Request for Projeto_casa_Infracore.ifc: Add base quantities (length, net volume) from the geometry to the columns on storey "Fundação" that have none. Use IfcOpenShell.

First a look at what the model holds.

```python
import ifcopenshell
import ifcopenshell.util.element
import ifcopenshell.util.unit

model = ifcopenshell.open("Projeto_casa_Infracore.ifc")
print(model.schema)
for unit_type in ("LENGTHUNIT", "AREAUNIT", "VOLUMEUNIT"):
    print(unit_type, ifcopenshell.util.unit.calculate_unit_scale(model, unit_type))
storey = next(s for s in model.by_type("IfcBuildingStorey") if s.Name == "Fundação")
columns = [e for e in ifcopenshell.util.element.get_decomposition(storey) if e.is_a("IfcColumn")]
for e in sorted(columns, key=lambda e: e.id()):
    print(e.id(), e.is_a(), e.Name, list(ifcopenshell.util.element.get_psets(e, qtos_only=True)), sep=" | ")
```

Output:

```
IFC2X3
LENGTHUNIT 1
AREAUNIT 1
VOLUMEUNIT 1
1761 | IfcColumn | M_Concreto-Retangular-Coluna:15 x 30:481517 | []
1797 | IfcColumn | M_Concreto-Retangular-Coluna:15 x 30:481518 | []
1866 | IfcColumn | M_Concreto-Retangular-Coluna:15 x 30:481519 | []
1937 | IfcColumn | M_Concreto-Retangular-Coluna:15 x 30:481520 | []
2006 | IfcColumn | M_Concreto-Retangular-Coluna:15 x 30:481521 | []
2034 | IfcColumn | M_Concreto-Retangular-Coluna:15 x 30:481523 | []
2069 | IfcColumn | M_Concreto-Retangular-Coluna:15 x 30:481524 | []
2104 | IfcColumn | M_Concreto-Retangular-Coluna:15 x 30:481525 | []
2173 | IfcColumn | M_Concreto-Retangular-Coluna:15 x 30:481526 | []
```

```python
import ifcopenshell
import ifcopenshell.api.pset
import ifcopenshell.geom
import ifcopenshell.util.element
import ifcopenshell.util.shape
import ifcopenshell.util.unit

model = ifcopenshell.open("Projeto_casa_Infracore.ifc")
unit_scale = ifcopenshell.util.unit.calculate_unit_scale(model)
volume_scale = ifcopenshell.util.unit.calculate_unit_scale(model, "VOLUMEUNIT")
settings = ifcopenshell.geom.settings()

storey = next(s for s in model.by_type("IfcBuildingStorey") if s.Name == "Fundação")
columns = [e for e in ifcopenshell.util.element.get_decomposition(storey) if e.is_a("IfcColumn")]

for e in sorted(columns, key=lambda e: e.id()):
    if ifcopenshell.util.element.get_psets(e, qtos_only=True, should_inherit=False):
        continue
    # Geometry comes back in metres, in the element's own axes.
    shape = ifcopenshell.geom.create_shape(settings, e)
    values = {
        "Length": ifcopenshell.util.shape.get_z(shape.geometry) / unit_scale,
        "NetVolume": ifcopenshell.util.shape.get_volume(shape.geometry) / volume_scale,
    }
    qto = ifcopenshell.api.pset.add_qto(model, product=e, name="BaseQuantities")
    ifcopenshell.api.pset.edit_qto(model, qto=qto, properties=values)
    print(e.id(), {k: round(v, 3) for k, v in values.items()})

model.write("Projeto_casa_Infracore_updated.ifc")
```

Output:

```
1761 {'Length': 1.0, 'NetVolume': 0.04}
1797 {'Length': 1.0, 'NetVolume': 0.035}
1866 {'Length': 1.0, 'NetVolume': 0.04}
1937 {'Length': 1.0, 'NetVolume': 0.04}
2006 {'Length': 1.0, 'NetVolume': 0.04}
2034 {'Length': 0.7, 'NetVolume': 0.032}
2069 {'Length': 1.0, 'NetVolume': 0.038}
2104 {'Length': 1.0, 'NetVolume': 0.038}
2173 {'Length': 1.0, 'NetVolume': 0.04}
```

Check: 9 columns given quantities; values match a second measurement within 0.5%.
